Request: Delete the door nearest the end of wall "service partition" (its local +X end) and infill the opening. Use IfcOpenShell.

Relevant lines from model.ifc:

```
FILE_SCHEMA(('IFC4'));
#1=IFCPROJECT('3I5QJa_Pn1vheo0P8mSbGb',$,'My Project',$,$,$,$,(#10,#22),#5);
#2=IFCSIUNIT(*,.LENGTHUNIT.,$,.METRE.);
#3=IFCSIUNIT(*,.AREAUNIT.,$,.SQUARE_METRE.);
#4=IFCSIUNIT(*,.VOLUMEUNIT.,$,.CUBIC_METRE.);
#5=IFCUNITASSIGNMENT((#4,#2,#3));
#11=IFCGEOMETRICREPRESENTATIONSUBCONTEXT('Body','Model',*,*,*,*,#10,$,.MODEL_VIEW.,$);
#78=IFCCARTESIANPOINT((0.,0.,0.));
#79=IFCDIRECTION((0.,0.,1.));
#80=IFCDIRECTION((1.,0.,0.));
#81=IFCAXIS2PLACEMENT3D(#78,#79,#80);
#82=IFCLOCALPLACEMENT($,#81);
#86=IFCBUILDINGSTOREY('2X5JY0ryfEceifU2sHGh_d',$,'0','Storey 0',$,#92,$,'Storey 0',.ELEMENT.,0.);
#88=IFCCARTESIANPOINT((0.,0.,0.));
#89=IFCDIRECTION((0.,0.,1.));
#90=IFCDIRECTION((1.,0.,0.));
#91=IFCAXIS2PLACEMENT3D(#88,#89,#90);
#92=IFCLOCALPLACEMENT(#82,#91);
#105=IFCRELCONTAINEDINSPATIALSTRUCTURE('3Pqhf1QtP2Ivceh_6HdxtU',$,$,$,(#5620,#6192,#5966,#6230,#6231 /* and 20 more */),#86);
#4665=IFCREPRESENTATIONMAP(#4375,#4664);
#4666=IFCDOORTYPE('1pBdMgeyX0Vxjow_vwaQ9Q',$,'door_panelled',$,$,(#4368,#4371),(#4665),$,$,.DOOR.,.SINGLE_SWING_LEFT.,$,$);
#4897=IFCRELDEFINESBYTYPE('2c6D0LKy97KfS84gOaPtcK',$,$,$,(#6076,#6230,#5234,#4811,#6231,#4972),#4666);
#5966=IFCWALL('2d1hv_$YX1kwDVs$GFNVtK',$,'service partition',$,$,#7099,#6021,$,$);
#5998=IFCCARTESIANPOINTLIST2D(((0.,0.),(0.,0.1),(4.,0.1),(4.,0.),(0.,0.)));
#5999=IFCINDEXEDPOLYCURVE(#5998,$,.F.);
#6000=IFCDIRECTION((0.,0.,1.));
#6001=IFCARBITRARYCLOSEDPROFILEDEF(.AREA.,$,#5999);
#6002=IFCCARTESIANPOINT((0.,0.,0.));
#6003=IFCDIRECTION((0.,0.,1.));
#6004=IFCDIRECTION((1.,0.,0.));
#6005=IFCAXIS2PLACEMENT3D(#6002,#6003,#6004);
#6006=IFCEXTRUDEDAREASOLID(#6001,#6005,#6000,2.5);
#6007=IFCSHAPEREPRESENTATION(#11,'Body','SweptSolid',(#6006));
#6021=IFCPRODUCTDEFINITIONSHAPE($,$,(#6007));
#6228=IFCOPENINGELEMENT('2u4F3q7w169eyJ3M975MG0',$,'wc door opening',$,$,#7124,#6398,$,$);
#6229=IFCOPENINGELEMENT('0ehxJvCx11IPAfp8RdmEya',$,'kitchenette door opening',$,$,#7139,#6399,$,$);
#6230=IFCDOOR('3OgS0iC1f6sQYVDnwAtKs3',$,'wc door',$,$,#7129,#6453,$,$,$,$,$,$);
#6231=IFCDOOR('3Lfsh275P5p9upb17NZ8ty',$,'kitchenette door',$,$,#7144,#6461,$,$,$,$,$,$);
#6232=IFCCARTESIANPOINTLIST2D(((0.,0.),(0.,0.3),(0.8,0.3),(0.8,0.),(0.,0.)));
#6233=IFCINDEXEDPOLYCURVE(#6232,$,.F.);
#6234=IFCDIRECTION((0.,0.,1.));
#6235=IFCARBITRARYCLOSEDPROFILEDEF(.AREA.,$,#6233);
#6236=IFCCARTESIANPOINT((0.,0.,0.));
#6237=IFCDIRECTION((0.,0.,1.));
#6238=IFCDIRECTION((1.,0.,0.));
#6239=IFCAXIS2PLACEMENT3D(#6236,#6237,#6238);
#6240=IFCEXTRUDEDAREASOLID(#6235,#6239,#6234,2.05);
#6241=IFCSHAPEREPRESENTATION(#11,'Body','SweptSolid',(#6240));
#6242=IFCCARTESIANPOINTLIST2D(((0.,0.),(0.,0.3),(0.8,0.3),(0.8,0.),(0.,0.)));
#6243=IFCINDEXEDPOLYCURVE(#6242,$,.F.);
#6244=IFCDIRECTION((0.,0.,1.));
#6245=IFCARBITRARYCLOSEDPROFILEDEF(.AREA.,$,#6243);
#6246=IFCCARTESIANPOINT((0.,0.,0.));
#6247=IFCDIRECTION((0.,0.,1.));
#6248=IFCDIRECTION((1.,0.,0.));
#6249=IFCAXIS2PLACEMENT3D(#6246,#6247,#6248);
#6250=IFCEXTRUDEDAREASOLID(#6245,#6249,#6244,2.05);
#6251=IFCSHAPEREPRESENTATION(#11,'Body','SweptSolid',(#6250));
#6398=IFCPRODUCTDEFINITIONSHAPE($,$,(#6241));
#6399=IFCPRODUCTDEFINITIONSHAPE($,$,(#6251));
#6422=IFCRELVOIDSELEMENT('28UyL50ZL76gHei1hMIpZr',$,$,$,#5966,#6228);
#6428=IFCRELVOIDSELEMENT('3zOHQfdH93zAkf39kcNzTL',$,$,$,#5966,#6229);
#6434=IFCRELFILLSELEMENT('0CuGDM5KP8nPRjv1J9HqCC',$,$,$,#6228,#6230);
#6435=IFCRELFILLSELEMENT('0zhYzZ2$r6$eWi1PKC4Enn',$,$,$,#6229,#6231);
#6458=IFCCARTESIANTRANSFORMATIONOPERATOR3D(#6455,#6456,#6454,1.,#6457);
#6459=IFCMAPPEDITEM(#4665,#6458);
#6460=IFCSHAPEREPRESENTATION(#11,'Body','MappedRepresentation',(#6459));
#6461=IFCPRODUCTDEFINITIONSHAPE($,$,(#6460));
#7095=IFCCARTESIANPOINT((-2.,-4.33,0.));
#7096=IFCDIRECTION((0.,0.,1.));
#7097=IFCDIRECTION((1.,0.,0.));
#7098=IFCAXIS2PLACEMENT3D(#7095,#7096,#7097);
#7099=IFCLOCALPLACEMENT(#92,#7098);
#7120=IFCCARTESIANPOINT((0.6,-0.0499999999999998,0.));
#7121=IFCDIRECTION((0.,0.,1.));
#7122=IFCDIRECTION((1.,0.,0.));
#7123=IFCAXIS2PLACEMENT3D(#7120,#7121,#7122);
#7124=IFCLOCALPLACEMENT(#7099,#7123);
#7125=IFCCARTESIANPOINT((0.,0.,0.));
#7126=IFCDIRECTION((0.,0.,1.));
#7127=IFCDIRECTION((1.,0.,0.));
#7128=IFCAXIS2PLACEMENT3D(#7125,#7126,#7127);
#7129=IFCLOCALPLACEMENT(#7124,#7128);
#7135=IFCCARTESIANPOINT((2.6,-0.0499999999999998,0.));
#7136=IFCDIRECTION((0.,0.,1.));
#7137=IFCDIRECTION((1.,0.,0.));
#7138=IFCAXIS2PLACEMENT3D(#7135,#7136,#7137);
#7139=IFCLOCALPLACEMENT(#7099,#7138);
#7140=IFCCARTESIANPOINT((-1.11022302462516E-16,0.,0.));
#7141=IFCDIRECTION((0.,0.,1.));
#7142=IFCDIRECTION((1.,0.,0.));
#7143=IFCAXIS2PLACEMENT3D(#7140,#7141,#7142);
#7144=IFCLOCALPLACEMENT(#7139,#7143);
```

```python
import ifcopenshell
import ifcopenshell.api.feature
import ifcopenshell.api.root
import ifcopenshell.geom
import ifcopenshell.util.shape

model = ifcopenshell.open("model.ifc")
settings = ifcopenshell.geom.settings()


def volume(element):
    """Net volume in cubic metres, openings subtracted."""
    shape = ifcopenshell.geom.create_shape(settings, element)
    return ifcopenshell.util.shape.get_volume(shape.geometry)


door = model.by_guid("3Lfsh275P5p9upb17NZ8ty")
opening = door.FillsVoids[0].RelatingOpeningElement
wall = opening.VoidsElements[0].RelatingBuildingElement
before = volume(wall)

ifcopenshell.api.root.remove_product(model, product=door)
ifcopenshell.api.feature.remove_feature(model, feature=opening)

after = volume(wall)

print(f"wall volume {before:.3f} -> {after:.3f} m3")

model.write("model_rev.ifc")
```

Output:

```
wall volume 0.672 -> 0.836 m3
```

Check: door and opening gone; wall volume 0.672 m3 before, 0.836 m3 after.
